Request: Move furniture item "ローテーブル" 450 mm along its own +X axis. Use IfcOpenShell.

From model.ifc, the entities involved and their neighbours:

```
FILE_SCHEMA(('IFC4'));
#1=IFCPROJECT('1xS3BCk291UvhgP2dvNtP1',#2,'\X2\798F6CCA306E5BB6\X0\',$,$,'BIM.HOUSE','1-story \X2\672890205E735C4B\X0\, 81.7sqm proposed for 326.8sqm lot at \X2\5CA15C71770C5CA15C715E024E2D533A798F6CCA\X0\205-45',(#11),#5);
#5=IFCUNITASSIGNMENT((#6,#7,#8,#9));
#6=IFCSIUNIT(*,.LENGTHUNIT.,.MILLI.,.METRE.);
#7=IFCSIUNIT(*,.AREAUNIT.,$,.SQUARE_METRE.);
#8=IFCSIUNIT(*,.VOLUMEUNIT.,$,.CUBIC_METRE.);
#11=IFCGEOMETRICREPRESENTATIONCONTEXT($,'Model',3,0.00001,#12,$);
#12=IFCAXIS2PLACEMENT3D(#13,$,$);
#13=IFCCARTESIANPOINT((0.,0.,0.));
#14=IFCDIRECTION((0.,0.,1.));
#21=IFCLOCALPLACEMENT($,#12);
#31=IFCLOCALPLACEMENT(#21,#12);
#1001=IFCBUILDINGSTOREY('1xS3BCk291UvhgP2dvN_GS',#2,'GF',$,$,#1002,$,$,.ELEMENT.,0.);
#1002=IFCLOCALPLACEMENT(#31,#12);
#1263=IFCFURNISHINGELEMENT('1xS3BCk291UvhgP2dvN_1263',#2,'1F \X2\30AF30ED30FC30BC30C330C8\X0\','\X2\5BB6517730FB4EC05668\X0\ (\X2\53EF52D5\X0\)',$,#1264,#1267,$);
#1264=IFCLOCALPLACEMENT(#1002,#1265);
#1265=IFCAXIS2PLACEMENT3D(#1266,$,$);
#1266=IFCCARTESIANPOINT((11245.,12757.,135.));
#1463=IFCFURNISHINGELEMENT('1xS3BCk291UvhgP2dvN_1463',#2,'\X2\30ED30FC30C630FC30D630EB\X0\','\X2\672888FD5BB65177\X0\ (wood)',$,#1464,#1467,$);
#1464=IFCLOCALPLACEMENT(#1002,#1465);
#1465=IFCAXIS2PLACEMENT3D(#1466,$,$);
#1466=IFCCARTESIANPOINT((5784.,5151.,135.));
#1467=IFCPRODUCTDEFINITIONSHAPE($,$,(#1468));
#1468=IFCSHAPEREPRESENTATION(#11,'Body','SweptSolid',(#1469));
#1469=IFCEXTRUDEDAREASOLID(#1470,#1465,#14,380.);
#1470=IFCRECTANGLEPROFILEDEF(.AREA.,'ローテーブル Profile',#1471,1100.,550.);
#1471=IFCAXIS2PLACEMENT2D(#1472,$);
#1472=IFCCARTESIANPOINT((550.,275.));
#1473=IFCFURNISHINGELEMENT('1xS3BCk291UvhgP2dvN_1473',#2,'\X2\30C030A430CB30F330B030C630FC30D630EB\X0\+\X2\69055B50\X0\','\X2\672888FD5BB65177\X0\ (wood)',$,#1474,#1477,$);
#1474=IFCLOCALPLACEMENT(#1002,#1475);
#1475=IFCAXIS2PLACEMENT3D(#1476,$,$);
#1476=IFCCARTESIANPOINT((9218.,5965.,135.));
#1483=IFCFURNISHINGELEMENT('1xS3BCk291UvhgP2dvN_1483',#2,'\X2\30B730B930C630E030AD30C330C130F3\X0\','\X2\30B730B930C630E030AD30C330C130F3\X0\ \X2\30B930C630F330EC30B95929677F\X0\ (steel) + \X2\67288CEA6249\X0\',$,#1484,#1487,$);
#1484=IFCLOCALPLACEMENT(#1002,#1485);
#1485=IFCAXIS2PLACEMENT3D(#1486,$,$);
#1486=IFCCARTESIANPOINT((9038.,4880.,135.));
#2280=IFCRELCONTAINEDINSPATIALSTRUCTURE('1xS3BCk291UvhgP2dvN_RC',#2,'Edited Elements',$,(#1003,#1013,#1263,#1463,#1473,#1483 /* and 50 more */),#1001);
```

```python
import ifcopenshell
import ifcopenshell.api.geometry
import ifcopenshell.util.placement
import ifcopenshell.util.unit

model = ifcopenshell.open("model.ifc")
unit_scale = ifcopenshell.util.unit.calculate_unit_scale(model)

item = model.by_guid("1xS3BCk291UvhgP2dvN_1463")
matrix = ifcopenshell.util.placement.get_local_placement(item.ObjectPlacement)
matrix[:3, 3] += matrix[:3, 0] * 0.45 / unit_scale
ifcopenshell.api.geometry.edit_object_placement(model, product=item, matrix=matrix, is_si=False)

print(ifcopenshell.util.placement.get_local_placement(item.ObjectPlacement).round(3) + 0.0)

model.write("model_updated.ifc")
```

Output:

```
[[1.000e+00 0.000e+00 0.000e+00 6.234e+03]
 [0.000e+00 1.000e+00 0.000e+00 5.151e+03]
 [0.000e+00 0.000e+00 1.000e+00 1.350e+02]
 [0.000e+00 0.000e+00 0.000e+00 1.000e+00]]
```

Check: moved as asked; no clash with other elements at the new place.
